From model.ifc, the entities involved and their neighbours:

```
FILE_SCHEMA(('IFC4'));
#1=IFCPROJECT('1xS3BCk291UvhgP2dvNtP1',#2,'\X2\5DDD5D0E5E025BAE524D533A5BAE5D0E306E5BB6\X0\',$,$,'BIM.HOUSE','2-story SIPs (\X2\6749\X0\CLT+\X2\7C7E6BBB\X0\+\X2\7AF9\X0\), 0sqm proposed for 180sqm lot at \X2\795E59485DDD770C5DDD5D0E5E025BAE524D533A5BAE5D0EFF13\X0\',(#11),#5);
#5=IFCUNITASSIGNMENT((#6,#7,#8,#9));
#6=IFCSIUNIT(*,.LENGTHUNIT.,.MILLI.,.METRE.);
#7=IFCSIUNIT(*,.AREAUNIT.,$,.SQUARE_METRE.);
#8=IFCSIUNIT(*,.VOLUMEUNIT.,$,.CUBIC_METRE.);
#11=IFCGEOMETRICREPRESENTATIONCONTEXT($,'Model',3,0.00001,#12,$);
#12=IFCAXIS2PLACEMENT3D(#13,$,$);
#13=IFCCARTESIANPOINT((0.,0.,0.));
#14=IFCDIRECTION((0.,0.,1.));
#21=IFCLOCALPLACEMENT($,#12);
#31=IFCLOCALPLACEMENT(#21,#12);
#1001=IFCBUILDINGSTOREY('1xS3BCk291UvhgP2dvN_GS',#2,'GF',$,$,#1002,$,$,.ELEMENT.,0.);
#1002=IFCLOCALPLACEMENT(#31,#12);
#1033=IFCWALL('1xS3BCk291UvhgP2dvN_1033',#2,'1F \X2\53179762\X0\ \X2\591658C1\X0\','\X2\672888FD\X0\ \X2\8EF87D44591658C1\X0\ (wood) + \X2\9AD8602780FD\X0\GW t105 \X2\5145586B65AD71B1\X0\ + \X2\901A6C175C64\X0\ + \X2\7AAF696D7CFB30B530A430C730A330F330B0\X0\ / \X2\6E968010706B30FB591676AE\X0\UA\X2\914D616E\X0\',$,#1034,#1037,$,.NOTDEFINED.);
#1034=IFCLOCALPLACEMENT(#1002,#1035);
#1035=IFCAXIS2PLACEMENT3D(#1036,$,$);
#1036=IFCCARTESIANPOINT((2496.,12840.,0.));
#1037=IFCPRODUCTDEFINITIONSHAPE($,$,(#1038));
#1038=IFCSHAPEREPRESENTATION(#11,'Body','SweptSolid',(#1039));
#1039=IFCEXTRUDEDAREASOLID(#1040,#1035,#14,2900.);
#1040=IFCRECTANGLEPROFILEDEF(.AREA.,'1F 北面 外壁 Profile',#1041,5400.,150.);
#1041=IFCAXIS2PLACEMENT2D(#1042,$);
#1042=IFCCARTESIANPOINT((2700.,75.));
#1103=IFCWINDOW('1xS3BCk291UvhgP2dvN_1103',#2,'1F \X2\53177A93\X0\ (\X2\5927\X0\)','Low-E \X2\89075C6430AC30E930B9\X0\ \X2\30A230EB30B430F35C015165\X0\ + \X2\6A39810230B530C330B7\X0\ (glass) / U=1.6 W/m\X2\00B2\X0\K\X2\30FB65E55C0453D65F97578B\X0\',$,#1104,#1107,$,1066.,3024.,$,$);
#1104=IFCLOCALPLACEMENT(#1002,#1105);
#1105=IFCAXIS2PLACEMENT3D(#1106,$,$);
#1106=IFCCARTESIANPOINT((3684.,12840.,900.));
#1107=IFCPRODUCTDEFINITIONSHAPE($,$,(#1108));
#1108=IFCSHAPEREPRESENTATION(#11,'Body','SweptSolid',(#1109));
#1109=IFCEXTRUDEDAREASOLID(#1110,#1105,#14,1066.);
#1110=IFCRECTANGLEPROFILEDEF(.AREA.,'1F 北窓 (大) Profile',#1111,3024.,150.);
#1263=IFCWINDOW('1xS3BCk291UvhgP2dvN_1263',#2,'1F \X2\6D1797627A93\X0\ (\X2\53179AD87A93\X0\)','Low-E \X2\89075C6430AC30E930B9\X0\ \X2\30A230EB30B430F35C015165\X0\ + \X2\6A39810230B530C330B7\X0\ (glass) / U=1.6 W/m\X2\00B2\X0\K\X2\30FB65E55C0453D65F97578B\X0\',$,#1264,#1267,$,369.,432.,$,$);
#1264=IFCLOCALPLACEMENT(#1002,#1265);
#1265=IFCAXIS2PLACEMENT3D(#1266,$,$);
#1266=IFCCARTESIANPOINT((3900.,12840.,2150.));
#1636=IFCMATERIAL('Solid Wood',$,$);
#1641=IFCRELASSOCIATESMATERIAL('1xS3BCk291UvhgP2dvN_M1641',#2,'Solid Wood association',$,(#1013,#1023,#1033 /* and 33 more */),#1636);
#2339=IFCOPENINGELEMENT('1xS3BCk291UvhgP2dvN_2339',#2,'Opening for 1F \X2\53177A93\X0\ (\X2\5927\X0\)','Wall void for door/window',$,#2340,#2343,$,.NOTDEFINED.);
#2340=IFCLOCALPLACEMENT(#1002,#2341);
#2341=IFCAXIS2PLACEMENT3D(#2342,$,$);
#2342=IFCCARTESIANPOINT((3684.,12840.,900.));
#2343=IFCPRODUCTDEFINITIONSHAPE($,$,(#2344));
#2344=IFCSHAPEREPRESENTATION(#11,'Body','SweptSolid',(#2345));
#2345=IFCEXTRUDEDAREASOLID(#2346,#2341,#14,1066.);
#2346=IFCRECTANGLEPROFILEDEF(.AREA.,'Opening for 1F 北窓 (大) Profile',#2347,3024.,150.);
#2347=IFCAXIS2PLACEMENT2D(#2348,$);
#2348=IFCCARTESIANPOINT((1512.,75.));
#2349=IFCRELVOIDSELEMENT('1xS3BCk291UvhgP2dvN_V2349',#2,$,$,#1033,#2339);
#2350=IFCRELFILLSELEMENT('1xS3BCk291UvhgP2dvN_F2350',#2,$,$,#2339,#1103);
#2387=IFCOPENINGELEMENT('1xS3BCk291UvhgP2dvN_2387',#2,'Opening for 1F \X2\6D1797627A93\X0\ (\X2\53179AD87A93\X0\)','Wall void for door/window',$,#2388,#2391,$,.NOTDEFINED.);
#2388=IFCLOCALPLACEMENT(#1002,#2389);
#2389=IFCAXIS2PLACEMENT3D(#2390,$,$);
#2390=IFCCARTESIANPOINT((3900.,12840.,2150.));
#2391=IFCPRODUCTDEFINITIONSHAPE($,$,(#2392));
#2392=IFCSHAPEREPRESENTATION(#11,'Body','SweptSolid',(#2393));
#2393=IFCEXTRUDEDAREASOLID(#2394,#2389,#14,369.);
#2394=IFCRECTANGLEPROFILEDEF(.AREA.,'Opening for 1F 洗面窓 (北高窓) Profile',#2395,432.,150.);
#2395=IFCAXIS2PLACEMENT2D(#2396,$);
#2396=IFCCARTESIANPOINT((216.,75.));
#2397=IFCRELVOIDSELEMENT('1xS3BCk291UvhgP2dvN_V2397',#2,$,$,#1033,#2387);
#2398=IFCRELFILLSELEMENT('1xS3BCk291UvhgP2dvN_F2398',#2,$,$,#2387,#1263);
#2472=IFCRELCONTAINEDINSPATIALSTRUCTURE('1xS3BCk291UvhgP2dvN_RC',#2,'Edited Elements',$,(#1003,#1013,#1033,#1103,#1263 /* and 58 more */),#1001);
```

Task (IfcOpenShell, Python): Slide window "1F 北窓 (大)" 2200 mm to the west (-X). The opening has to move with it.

```python
import ifcopenshell
import ifcopenshell.api.geometry
import ifcopenshell.util.placement

model = ifcopenshell.open("model.ifc")

window = model.by_guid("1xS3BCk291UvhgP2dvN_1103")
opening = window.FillsVoids[0].RelatingOpeningElement
wall = opening.VoidsElements[0].RelatingBuildingElement

wall_matrix = ifcopenshell.util.placement.get_local_placement(wall.ObjectPlacement)
shift = wall_matrix[:3, 0] * -2200.0
before = ifcopenshell.util.placement.get_local_placement(window.ObjectPlacement)[:3, 3].copy()

# The window is not placed relative to its opening, so move both.
for product in (opening, window):
    matrix = ifcopenshell.util.placement.get_local_placement(product.ObjectPlacement)
    matrix[:3, 3] += shift
    ifcopenshell.api.geometry.edit_object_placement(model, product=product, matrix=matrix, is_si=False)

after = ifcopenshell.util.placement.get_local_placement(window.ObjectPlacement)[:3, 3]
print("window moved by", (after - before).round(3) + 0.0)

model.write("model_v2.ifc")
```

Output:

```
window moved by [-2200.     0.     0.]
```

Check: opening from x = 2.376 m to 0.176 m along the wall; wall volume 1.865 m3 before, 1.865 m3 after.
